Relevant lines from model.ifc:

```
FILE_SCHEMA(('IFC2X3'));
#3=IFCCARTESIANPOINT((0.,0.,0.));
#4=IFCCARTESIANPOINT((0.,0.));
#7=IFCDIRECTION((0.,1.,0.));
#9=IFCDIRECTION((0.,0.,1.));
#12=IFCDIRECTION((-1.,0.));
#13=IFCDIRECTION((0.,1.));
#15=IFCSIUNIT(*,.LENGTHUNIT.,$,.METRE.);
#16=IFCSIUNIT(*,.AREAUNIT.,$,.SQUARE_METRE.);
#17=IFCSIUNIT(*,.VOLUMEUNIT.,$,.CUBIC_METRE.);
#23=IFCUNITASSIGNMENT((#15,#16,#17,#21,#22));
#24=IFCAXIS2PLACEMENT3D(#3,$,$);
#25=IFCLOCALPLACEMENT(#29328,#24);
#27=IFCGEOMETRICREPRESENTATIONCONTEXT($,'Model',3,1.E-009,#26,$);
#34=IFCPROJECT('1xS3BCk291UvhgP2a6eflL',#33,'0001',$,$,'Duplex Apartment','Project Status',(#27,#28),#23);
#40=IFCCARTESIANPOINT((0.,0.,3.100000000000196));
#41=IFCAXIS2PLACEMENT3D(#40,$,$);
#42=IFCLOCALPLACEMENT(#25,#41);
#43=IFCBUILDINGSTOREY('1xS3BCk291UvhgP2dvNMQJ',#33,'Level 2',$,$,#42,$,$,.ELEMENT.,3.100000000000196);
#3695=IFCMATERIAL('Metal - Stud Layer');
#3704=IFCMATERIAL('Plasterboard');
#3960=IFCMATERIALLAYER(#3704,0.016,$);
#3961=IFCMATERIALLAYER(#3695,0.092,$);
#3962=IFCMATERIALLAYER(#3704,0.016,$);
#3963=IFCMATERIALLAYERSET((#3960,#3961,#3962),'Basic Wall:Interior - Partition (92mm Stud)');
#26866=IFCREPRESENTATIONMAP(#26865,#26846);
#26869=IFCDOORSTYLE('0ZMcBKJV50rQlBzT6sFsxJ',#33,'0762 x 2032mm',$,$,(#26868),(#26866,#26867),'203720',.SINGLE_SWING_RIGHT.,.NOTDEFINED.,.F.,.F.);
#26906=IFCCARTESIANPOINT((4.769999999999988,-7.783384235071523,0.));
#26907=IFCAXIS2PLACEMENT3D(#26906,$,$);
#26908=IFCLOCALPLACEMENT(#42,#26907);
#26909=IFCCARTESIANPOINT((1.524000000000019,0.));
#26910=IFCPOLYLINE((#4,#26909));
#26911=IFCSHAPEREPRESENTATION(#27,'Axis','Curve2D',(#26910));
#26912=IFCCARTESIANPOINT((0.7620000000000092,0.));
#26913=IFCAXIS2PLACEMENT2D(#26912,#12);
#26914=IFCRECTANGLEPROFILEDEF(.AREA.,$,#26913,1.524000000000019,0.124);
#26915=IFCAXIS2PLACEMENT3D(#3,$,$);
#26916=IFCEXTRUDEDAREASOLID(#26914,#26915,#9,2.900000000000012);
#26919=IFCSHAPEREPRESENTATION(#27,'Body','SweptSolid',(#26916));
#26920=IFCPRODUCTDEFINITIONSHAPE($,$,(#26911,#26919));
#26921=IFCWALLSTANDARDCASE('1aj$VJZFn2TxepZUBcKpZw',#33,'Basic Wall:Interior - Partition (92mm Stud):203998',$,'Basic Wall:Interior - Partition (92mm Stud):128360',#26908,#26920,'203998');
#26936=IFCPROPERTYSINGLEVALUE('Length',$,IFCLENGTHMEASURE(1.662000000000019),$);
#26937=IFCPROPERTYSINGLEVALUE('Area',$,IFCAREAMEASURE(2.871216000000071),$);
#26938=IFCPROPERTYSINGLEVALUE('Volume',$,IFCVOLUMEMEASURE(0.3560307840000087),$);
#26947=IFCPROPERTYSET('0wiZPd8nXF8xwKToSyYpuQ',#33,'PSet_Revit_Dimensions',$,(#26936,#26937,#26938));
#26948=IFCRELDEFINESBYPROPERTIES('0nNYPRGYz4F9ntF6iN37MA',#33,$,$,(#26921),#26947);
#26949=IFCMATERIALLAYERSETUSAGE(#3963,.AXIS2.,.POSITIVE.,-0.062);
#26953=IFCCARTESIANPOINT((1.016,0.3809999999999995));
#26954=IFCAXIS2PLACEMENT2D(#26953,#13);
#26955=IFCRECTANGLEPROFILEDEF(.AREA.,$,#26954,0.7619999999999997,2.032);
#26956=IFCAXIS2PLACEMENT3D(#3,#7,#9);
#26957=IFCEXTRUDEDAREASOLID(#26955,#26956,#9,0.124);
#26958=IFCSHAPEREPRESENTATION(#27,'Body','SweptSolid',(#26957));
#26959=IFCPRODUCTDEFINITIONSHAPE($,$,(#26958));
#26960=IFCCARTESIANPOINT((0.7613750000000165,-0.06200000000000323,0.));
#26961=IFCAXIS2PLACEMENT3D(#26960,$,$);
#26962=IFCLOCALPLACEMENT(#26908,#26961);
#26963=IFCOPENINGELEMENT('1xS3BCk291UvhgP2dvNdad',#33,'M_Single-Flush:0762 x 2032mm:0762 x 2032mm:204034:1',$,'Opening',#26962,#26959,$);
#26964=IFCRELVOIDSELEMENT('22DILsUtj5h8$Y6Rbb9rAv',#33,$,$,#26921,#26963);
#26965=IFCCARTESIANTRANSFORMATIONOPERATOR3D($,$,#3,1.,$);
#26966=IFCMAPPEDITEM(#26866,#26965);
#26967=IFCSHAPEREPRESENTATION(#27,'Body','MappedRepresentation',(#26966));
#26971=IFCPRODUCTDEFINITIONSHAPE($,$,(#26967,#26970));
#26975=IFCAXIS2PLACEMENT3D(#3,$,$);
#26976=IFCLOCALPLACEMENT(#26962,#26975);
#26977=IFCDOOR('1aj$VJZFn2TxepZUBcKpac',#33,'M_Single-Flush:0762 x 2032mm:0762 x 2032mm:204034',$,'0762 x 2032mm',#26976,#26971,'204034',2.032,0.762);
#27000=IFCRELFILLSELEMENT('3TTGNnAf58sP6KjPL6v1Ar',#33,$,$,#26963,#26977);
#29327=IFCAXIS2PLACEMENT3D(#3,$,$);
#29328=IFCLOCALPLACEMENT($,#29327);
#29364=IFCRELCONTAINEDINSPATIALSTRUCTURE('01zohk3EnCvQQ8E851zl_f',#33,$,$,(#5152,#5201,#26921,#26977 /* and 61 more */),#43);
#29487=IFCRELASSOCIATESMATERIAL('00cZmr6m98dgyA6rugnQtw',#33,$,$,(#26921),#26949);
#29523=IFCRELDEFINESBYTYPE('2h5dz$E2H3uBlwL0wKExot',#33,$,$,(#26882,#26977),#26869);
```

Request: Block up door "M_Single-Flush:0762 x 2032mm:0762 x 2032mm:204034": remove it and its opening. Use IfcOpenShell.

```python
import ifcopenshell
import ifcopenshell.api.feature
import ifcopenshell.api.pset
import ifcopenshell.api.root
import ifcopenshell.geom
import ifcopenshell.util.element
import ifcopenshell.util.shape
import ifcopenshell.util.unit

model = ifcopenshell.open("model.ifc")
area_scale = ifcopenshell.util.unit.calculate_unit_scale(model, "AREAUNIT")
volume_scale = ifcopenshell.util.unit.calculate_unit_scale(model, "VOLUMEUNIT")
settings = ifcopenshell.geom.settings()


def volume(element):
    """Net volume in cubic metres, openings subtracted."""
    shape = ifcopenshell.geom.create_shape(settings, element)
    return ifcopenshell.util.shape.get_volume(shape.geometry)


door = model.by_guid("1aj$VJZFn2TxepZUBcKpac")
opening = door.FillsVoids[0].RelatingOpeningElement
wall = opening.VoidsElements[0].RelatingBuildingElement
before = volume(wall)

ifcopenshell.api.root.remove_product(model, product=door)
ifcopenshell.api.feature.remove_feature(model, feature=opening)

after = volume(wall)
thickness = 0.124  # wall thickness in metres

# Update the wall's stored quantities.
pset = model.by_id(ifcopenshell.util.element.get_pset(wall, "PSet_Revit_Dimensions", should_inherit=False)["id"])
ifcopenshell.api.pset.edit_pset(model, pset=pset, properties={
    "Area": model.create_entity("IfcAreaMeasure", after / thickness / area_scale),
    "Volume": model.create_entity("IfcVolumeMeasure", after / volume_scale),
})

print(f"wall volume {before:.3f} -> {after:.3f} m3")

model.write("model_edited.ifc")
```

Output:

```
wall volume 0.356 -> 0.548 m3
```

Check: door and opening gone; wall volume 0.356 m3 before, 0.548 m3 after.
